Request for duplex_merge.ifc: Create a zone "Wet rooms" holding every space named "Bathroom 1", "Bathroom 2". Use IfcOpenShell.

First a look at what the model holds.

```python
import ifcopenshell

model = ifcopenshell.open("duplex_merge.ifc")
print(model.schema)
seen = {}
for space in model.by_type("IfcSpace"):
    seen[space.LongName] = seen.get(space.LongName, 0) + 1
for name, count in sorted(seen.items(), key=str):
    print(count, "x", name)
print("zones:", [z.Name for z in model.by_type("IfcZone")][:20])
```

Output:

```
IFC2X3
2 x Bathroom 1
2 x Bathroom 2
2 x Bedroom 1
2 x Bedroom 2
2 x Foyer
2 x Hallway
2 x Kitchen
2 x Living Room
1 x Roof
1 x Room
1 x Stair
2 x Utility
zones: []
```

```python
import ifcopenshell
import ifcopenshell.api.group
import ifcopenshell.api.root

model = ifcopenshell.open("duplex_merge.ifc")

names = {"Bathroom 1", "Bathroom 2"}
spaces = [s for s in model.by_type("IfcSpace") if s.LongName in names]

zone = ifcopenshell.api.root.create_entity(model, ifc_class="IfcZone", name="Wet rooms")
ifcopenshell.api.group.assign_group(model, products=spaces, group=zone)
print(len(spaces), "spaces in", zone.Name)

model.write("duplex_merge_edited.ifc")
```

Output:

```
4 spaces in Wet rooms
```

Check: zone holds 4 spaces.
